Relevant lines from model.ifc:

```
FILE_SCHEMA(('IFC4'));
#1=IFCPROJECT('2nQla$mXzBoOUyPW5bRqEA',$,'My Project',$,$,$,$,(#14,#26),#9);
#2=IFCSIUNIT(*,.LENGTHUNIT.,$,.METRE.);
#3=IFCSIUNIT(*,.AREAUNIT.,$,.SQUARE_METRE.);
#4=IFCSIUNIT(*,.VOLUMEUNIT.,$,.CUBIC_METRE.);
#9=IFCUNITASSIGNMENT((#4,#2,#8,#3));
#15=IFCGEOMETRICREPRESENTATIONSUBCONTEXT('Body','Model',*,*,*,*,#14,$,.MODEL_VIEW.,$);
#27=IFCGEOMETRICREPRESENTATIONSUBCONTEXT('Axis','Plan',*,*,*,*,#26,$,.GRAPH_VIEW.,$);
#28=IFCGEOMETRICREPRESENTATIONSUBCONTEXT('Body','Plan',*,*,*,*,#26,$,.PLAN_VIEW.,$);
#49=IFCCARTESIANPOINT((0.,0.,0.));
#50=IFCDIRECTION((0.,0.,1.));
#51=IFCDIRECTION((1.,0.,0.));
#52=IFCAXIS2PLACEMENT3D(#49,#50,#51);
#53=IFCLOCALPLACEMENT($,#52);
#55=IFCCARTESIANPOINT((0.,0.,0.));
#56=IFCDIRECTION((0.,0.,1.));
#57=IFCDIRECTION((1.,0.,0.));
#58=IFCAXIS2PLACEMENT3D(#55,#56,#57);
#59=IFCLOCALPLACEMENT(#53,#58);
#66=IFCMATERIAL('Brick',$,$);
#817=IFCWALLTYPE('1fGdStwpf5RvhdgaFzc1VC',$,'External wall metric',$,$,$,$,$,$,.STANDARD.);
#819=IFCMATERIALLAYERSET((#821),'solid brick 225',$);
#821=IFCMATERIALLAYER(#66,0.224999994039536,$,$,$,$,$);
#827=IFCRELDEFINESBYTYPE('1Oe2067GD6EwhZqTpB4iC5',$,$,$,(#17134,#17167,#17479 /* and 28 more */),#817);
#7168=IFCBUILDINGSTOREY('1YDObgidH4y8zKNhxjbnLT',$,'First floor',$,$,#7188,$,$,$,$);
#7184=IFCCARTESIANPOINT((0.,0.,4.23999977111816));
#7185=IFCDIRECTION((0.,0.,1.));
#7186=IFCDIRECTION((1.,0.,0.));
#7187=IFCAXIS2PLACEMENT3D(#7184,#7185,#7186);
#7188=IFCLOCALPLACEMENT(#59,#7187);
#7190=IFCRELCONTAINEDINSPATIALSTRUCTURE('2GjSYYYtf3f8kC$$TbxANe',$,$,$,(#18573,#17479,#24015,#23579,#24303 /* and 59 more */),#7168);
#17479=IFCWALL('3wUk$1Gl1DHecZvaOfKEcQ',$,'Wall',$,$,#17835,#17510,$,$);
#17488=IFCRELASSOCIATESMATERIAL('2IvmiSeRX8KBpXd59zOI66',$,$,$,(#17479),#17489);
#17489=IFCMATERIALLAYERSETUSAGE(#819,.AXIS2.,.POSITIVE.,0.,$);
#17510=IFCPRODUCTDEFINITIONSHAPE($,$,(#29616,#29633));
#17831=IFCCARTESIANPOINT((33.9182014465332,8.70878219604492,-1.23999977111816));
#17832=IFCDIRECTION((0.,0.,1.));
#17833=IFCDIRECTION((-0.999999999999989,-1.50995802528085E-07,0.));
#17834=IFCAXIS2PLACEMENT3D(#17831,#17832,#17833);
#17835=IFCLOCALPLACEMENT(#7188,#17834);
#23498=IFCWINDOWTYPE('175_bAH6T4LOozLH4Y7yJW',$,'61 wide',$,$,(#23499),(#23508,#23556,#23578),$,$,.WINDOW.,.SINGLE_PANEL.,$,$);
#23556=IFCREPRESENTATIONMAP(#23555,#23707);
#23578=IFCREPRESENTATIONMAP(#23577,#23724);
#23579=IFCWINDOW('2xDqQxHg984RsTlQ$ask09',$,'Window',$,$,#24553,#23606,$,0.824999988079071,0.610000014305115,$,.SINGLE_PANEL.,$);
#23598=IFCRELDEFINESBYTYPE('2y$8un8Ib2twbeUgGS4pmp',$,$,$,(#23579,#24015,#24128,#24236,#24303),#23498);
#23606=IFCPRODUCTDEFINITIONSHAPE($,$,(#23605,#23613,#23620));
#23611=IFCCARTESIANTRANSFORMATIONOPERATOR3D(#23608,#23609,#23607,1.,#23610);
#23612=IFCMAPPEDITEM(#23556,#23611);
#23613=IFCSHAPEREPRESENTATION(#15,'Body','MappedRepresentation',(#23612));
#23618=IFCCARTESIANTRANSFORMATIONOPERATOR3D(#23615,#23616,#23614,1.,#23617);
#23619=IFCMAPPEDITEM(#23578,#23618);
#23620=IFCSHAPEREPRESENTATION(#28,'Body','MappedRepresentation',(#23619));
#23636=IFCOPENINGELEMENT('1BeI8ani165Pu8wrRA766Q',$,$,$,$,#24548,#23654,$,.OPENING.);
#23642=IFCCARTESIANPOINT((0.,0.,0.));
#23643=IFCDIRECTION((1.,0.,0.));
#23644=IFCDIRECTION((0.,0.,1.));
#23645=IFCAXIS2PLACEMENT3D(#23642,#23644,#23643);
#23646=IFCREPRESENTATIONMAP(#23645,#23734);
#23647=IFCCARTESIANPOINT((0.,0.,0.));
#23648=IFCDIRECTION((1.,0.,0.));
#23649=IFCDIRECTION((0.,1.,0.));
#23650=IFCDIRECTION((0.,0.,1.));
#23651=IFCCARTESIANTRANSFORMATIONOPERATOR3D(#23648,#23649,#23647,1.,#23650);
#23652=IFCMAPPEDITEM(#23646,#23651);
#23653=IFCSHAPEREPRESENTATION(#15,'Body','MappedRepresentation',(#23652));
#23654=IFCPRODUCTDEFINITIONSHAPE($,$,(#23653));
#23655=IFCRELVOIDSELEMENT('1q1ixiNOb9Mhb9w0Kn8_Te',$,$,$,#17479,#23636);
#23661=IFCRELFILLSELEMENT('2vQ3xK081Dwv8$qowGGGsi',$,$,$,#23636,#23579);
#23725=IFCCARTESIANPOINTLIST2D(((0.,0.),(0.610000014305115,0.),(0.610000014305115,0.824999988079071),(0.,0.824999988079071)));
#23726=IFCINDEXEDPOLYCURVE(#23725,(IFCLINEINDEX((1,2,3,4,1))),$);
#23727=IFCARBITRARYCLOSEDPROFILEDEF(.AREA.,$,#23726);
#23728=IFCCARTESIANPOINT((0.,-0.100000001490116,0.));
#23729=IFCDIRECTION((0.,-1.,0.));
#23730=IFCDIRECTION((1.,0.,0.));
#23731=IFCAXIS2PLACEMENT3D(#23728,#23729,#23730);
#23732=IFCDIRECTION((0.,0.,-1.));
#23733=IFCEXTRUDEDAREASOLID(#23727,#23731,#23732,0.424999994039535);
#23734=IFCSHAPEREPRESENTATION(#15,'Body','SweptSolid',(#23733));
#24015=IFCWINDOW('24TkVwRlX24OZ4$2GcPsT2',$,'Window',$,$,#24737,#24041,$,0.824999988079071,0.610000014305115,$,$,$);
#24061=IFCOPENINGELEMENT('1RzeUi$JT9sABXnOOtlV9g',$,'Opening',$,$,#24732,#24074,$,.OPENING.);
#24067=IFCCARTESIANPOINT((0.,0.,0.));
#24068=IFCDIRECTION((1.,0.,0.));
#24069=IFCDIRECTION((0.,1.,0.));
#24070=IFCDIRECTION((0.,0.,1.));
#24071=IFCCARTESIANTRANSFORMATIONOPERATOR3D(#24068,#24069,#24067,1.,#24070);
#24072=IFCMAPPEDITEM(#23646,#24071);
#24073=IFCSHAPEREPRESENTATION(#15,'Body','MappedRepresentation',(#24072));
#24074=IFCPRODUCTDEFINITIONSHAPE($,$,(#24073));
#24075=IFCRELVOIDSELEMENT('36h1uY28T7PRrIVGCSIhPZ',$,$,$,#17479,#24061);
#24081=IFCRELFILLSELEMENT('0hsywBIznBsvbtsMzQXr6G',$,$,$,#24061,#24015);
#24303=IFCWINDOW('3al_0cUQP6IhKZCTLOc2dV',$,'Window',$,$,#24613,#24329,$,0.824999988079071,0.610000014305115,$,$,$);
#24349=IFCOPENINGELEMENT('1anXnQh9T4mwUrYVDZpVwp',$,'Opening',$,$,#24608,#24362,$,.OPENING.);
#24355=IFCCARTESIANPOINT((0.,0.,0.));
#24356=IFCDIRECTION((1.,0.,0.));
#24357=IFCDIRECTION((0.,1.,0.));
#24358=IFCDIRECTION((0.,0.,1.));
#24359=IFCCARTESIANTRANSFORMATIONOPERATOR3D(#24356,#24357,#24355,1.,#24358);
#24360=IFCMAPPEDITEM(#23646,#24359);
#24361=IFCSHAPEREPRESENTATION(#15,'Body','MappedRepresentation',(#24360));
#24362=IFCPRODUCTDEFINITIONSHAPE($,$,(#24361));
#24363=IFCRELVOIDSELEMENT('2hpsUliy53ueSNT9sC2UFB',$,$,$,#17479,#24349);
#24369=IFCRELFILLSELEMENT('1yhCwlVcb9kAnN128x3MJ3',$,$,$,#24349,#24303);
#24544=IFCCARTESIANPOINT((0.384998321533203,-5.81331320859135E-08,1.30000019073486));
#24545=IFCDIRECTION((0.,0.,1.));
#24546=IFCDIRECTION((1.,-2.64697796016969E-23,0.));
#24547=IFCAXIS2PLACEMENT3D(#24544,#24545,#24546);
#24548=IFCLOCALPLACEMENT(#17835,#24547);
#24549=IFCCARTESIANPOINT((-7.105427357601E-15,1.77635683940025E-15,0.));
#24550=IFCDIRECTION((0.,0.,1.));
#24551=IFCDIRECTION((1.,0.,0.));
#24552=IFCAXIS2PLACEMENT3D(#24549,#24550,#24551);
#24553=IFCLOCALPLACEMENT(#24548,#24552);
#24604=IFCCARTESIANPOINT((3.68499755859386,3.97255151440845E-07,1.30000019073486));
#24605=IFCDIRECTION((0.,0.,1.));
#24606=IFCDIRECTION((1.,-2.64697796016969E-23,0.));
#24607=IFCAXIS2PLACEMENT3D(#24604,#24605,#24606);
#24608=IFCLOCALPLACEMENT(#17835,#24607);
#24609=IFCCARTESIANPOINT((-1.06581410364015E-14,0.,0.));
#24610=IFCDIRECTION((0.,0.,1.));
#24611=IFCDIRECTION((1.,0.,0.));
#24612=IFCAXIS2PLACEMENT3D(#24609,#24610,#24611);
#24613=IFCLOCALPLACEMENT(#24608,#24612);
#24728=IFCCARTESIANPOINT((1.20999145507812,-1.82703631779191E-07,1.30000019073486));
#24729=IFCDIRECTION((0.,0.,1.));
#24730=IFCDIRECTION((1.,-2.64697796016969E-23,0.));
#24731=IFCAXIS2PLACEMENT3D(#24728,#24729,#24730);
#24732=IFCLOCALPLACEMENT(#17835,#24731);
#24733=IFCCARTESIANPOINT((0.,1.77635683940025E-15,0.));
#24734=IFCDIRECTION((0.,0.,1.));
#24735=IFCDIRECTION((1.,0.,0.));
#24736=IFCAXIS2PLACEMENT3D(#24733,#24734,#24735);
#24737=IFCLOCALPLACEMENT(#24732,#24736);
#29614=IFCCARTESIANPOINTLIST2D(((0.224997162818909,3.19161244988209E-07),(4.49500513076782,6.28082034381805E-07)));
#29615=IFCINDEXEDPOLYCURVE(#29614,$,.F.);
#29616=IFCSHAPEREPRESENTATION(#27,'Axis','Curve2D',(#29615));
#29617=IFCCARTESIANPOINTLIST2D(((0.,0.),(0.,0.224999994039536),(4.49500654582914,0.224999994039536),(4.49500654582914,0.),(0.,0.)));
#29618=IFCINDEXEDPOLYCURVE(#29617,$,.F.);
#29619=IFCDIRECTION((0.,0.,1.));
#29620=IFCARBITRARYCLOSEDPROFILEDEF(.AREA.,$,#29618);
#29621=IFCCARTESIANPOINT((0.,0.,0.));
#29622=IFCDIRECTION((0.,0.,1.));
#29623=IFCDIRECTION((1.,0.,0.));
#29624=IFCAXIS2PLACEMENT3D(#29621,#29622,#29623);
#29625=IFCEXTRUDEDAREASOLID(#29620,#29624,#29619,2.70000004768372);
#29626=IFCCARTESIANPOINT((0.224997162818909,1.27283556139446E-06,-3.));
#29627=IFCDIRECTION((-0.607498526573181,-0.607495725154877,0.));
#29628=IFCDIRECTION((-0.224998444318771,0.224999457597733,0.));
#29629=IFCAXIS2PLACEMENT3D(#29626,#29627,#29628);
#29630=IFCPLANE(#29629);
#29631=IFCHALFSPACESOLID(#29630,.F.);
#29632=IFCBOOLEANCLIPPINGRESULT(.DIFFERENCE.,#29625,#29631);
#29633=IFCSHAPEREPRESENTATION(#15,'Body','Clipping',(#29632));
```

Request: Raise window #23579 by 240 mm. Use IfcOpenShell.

```python
import numpy as np
import ifcopenshell
import ifcopenshell.api.geometry
import ifcopenshell.util.placement
import ifcopenshell.util.unit

model = ifcopenshell.open("model.ifc")
unit_scale = ifcopenshell.util.unit.calculate_unit_scale(model)

window = model.by_guid("2xDqQxHg984RsTlQ$ask09")
opening = window.FillsVoids[0].RelatingOpeningElement
dz = 0.24 / unit_scale

shift = np.array([0.0, 0.0, dz])
# The window is placed relative to its opening, so it follows when the opening moves.
matrix = ifcopenshell.util.placement.get_local_placement(opening.ObjectPlacement)
matrix[:3, 3] += shift
ifcopenshell.api.geometry.edit_object_placement(
    model, product=opening, matrix=matrix, is_si=False, should_transform_children=True
)

print(f"moved by {dz * unit_scale:+.3f} m")

model.write("model_updated.ifc")
```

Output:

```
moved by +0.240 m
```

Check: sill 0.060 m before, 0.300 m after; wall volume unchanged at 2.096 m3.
